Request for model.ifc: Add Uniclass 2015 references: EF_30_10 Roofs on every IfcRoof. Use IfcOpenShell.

First a look at what the model holds.

```python
import ifcopenshell

model = ifcopenshell.open("model.ifc")
print(model.schema)
print("classifications:", [c.Name for c in model.by_type("IfcClassification")])
for ifc_class in ("IfcDoor", "IfcRoof", "IfcStair", "IfcWall", "IfcWindow"):
    print(ifc_class, len(model.by_type(ifc_class)))
```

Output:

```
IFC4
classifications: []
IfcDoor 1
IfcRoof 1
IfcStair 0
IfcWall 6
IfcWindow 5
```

```python
import ifcopenshell
import ifcopenshell.api.classification

model = ifcopenshell.open("model.ifc")

system = ifcopenshell.api.classification.add_classification(model, classification="Uniclass 2015")

codes = {
    "IfcRoof": ("EF_30_10", "Roofs"),
}
for ifc_class, (code, name) in codes.items():
    products = model.by_type(ifc_class)
    ifcopenshell.api.classification.add_reference(
        model, products=products, classification=system, identification=code, name=name
    )
    print(code, len(products))

model.write("model-out.ifc")
```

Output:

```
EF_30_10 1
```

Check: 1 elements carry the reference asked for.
